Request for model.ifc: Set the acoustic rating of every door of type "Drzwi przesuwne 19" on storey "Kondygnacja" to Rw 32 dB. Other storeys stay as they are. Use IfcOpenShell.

First a look at what the model holds.

```python
import ifcopenshell
import ifcopenshell.util.element

model = ifcopenshell.open("model.ifc")
print(model.schema)
storey = next(s for s in model.by_type("IfcBuildingStorey") if s.Name == "Kondygnacja")
doors = [e for e in ifcopenshell.util.element.get_decomposition(storey) if e.is_a("IfcDoor")]
seen = {}
for e in doors:
    element_type = ifcopenshell.util.element.get_type(e)
    key = (element_type.Name if element_type != e and element_type else None, ifcopenshell.util.element.get_pset(e, "Pset_DoorCommon", "AcousticRating"))
    seen[key] = seen.get(key, 0) + 1
for (name, value), count in sorted(seen.items(), key=str):
    print(count, "x", name, "|", value)
```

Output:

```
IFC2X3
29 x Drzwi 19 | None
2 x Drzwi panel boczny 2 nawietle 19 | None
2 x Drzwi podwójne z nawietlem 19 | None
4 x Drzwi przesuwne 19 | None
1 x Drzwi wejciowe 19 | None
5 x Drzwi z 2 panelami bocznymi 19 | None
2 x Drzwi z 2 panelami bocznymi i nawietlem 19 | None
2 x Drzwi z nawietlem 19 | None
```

```python
import ifcopenshell
import ifcopenshell.api.pset
import ifcopenshell.util.element

model = ifcopenshell.open("model.ifc")

storey = next(s for s in model.by_type("IfcBuildingStorey") if s.Name == "Kondygnacja")
doors = [e for e in ifcopenshell.util.element.get_decomposition(storey) if e.is_a("IfcDoor")]

count = 0
for e in doors:
    element_type = ifcopenshell.util.element.get_type(e)
    if element_type in (None, e) or element_type.Name != "Drzwi przesuwne 19":
        continue
    # add_pset returns the element's existing set when there is one.
    pset = ifcopenshell.api.pset.add_pset(model, product=e, name="Pset_DoorCommon")
    ifcopenshell.api.pset.edit_pset(model, pset=pset, properties={"AcousticRating": "Rw 32 dB"})
    count += 1

print(count, "doors updated")

model.write("model_rev.ifc")
```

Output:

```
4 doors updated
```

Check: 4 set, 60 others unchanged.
